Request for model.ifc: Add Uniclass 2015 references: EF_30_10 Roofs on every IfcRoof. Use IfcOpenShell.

First a look at what the model holds.

```python
import ifcopenshell

model = ifcopenshell.open("model.ifc")
print(model.schema)
print("classifications:", [c.Name for c in model.by_type("IfcClassification")])
for ifc_class in ("IfcDoor", "IfcRoof", "IfcStair", "IfcWall", "IfcWindow"):
    print(ifc_class, len(model.by_type(ifc_class)))
```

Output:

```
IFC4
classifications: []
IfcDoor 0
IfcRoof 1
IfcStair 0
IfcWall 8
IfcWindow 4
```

```python
import ifcopenshell
import ifcopenshell.api.classification

model = ifcopenshell.open("model.ifc")

system = ifcopenshell.api.classification.add_classification(model, classification="Uniclass 2015")

codes = {
    "IfcRoof": ("EF_30_10", "Roofs"),
}
for ifc_class, (code, name) in codes.items():
    products = model.by_type(ifc_class)
    ifcopenshell.api.classification.add_reference(
        model, products=products, classification=system, identification=code, name=name
    )
    print(code, len(products))

model.write("model-out.ifc")
```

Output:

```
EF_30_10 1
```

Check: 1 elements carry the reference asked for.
